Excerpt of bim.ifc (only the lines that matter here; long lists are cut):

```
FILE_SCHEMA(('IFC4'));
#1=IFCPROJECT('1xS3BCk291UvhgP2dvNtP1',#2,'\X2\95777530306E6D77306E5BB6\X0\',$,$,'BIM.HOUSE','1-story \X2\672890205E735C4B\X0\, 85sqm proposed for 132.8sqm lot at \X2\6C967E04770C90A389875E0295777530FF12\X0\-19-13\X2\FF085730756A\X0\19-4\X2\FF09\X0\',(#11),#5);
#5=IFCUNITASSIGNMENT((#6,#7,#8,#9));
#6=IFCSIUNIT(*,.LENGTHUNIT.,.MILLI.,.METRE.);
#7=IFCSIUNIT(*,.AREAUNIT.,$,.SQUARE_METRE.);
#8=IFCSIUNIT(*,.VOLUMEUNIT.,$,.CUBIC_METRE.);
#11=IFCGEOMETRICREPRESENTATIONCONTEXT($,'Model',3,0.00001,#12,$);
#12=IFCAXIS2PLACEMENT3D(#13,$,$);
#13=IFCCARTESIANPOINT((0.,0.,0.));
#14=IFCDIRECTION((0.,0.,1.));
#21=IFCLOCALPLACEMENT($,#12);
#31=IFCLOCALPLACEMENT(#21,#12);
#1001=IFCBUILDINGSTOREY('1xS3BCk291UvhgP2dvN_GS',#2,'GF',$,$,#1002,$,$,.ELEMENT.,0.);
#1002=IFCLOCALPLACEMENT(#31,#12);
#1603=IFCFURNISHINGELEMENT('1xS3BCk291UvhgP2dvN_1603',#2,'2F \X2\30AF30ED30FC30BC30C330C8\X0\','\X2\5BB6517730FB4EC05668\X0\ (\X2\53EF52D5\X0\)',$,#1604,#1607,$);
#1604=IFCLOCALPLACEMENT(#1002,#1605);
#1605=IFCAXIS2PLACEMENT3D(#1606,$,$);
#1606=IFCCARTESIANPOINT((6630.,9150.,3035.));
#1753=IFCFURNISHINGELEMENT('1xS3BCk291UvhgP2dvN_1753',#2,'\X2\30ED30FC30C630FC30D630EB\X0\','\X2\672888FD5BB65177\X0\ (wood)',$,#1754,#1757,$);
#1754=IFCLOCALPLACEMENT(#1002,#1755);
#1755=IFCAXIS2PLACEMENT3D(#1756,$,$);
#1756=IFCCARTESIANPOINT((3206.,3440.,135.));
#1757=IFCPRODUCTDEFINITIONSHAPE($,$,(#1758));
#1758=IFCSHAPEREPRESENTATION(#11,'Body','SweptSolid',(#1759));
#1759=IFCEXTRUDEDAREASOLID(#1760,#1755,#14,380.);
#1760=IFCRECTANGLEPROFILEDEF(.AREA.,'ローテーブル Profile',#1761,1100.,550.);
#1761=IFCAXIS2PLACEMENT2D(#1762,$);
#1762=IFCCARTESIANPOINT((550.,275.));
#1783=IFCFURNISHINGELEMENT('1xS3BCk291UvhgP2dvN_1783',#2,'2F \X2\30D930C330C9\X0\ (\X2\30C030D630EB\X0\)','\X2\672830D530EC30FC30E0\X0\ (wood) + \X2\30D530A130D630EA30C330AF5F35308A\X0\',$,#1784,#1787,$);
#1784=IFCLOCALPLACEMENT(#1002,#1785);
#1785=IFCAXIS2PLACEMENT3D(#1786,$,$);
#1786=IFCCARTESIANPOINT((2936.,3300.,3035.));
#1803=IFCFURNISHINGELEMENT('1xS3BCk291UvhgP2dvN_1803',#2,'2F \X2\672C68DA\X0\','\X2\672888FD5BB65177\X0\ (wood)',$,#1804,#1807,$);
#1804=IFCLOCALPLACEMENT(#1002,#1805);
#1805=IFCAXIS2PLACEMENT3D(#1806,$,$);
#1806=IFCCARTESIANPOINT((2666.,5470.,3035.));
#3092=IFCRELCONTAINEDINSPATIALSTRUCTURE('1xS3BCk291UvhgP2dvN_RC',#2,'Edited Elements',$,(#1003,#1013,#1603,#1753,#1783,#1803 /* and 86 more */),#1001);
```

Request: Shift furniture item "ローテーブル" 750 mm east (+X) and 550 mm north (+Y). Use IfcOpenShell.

```python
import ifcopenshell
import ifcopenshell.api.geometry
import ifcopenshell.util.placement

model = ifcopenshell.open("bim.ifc")

item = model.by_id(1753)
matrix = ifcopenshell.util.placement.get_local_placement(item.ObjectPlacement)
matrix[0, 3] += 750.0
matrix[1, 3] += 550.0
ifcopenshell.api.geometry.edit_object_placement(model, product=item, matrix=matrix, is_si=False)

print(ifcopenshell.util.placement.get_local_placement(item.ObjectPlacement).round(3) + 0.0)

model.write("bim_v2.ifc")
```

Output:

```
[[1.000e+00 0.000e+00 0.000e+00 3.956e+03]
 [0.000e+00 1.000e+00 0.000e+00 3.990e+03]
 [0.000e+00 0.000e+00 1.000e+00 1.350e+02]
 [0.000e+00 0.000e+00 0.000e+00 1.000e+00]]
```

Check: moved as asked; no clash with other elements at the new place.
